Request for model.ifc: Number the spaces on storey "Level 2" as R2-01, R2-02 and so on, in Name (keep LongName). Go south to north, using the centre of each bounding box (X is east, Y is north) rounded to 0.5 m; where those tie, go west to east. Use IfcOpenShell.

First a look at what the model holds.

```python
import ifcopenshell
import ifcopenshell.util.element
import ifcopenshell.util.placement

model = ifcopenshell.open("model.ifc")
print(model.schema)
storey = next(s for s in model.by_type("IfcBuildingStorey") if s.Name == "Level 2")
spaces = [e for e in ifcopenshell.util.element.get_decomposition(storey) if e.is_a("IfcSpace")]
for e in sorted(spaces, key=lambda e: e.id()):
    origin = ifcopenshell.util.placement.get_local_placement(e.ObjectPlacement)[:3, 3]
    print(e.id(), e.Name, e.LongName, origin.round(2) + 0.0, sep=" | ")
```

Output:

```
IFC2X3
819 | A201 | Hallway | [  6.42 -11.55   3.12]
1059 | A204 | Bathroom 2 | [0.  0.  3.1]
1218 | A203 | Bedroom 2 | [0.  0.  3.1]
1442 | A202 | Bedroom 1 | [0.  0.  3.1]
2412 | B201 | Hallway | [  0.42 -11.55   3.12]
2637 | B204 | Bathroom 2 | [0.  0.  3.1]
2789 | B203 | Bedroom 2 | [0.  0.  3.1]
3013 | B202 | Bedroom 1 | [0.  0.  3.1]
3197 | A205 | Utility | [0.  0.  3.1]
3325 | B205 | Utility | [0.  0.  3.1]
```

```python
import ifcopenshell
import ifcopenshell.geom
import ifcopenshell.util.element
import ifcopenshell.util.shape

model = ifcopenshell.open("model.ifc")
settings = ifcopenshell.geom.settings()
settings.set("use-world-coords", True)


def centre(element):
    shape = ifcopenshell.geom.create_shape(settings, element)
    return ifcopenshell.util.shape.get_bbox_centroid(shape.geometry)


storey = next(s for s in model.by_type("IfcBuildingStorey") if s.Name == "Level 2")
spaces = [e for e in ifcopenshell.util.element.get_decomposition(storey) if e.is_a("IfcSpace")]

# Insertion points can sit at a corner or the storey origin, so sort by the geometry (in metres).
centres = {e: centre(e) for e in spaces}
spaces.sort(key=lambda e: (round(centres[e][1] / 0.5), centres[e][0]))

for i, e in enumerate(spaces, start=1):
    number = f"R2-{i:02d}"
    e.Name = number
    print(e.id(), number)

model.write("model_updated.ifc")
```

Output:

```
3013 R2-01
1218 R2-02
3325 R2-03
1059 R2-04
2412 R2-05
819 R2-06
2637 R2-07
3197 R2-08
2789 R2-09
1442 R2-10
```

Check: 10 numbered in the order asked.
